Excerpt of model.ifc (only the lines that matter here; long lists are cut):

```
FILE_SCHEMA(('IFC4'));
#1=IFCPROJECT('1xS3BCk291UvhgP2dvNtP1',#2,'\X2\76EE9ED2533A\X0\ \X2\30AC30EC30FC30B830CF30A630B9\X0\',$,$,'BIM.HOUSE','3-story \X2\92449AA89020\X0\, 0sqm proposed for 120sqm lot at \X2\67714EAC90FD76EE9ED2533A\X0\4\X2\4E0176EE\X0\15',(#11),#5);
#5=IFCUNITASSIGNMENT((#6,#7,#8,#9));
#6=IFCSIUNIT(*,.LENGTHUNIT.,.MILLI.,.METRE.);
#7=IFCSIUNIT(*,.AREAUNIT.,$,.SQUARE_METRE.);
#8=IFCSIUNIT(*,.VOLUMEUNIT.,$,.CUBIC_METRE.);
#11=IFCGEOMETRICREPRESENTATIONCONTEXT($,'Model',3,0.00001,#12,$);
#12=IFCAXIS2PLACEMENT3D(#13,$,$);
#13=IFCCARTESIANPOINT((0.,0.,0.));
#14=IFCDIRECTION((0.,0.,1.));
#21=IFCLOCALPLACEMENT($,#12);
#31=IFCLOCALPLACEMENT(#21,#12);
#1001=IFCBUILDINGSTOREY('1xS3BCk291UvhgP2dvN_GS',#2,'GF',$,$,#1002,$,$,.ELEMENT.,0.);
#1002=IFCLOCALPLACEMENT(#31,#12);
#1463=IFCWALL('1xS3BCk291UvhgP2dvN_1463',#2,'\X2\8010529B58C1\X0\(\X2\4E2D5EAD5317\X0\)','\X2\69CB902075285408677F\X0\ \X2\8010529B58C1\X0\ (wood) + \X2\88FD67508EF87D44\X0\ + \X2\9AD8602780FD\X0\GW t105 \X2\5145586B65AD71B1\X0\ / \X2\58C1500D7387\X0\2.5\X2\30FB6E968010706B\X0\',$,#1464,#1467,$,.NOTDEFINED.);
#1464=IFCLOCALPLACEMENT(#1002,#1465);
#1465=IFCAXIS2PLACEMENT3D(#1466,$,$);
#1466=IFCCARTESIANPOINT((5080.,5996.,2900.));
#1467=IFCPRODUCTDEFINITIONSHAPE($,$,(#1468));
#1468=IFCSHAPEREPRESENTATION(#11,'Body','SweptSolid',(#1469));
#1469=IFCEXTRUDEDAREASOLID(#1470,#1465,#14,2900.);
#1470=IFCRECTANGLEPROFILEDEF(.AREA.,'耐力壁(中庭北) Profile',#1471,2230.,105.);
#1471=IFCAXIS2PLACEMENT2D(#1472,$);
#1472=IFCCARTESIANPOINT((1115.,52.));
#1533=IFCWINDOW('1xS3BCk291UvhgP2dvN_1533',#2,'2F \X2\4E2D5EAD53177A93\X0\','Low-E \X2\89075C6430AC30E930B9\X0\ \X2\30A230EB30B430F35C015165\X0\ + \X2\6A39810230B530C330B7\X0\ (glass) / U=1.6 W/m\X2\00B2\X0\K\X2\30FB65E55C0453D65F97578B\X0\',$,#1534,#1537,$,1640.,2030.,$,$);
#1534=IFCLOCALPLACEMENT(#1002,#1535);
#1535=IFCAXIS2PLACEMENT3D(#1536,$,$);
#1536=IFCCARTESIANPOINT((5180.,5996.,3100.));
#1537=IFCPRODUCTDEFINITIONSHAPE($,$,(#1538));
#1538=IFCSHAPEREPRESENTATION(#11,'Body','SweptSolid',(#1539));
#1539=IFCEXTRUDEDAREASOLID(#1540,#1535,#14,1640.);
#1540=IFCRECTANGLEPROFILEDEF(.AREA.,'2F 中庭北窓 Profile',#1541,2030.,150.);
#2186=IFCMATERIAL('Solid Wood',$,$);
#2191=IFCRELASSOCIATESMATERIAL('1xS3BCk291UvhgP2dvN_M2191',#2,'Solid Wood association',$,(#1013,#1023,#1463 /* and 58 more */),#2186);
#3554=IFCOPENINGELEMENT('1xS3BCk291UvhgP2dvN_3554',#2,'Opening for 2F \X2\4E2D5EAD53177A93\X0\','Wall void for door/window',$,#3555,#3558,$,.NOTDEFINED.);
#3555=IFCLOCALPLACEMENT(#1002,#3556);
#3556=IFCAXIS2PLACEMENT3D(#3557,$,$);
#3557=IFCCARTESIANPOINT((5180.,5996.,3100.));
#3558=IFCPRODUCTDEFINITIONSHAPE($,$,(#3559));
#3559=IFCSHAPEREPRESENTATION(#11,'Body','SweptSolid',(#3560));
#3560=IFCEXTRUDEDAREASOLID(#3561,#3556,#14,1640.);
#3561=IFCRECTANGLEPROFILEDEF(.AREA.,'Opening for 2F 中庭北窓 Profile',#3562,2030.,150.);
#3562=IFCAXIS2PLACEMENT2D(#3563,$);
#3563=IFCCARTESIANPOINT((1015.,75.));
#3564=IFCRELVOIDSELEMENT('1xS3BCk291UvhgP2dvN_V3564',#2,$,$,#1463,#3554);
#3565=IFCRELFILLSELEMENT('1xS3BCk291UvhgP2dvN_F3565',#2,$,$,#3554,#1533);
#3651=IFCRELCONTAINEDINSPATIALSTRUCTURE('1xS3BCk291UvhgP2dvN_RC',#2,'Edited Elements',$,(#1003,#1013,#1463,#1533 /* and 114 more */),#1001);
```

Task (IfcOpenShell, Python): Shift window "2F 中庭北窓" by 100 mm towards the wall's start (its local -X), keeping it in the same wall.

```python
import ifcopenshell
import ifcopenshell.api.geometry
import ifcopenshell.util.placement

model = ifcopenshell.open("model.ifc")

window = model.by_guid("1xS3BCk291UvhgP2dvN_1533")
opening = window.FillsVoids[0].RelatingOpeningElement
wall = opening.VoidsElements[0].RelatingBuildingElement

wall_matrix = ifcopenshell.util.placement.get_local_placement(wall.ObjectPlacement)
shift = wall_matrix[:3, 0] * -100.0
before = ifcopenshell.util.placement.get_local_placement(window.ObjectPlacement)[:3, 3].copy()

# The window is not placed relative to its opening, so move both.
for product in (opening, window):
    matrix = ifcopenshell.util.placement.get_local_placement(product.ObjectPlacement)
    matrix[:3, 3] += shift
    ifcopenshell.api.geometry.edit_object_placement(model, product=product, matrix=matrix, is_si=False)

after = ifcopenshell.util.placement.get_local_placement(window.ObjectPlacement)[:3, 3]
print("window moved by", (after - before).round(3) + 0.0)

model.write("model-out.ifc")
```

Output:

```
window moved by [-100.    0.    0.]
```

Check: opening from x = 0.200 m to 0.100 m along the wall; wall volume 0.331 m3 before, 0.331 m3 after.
